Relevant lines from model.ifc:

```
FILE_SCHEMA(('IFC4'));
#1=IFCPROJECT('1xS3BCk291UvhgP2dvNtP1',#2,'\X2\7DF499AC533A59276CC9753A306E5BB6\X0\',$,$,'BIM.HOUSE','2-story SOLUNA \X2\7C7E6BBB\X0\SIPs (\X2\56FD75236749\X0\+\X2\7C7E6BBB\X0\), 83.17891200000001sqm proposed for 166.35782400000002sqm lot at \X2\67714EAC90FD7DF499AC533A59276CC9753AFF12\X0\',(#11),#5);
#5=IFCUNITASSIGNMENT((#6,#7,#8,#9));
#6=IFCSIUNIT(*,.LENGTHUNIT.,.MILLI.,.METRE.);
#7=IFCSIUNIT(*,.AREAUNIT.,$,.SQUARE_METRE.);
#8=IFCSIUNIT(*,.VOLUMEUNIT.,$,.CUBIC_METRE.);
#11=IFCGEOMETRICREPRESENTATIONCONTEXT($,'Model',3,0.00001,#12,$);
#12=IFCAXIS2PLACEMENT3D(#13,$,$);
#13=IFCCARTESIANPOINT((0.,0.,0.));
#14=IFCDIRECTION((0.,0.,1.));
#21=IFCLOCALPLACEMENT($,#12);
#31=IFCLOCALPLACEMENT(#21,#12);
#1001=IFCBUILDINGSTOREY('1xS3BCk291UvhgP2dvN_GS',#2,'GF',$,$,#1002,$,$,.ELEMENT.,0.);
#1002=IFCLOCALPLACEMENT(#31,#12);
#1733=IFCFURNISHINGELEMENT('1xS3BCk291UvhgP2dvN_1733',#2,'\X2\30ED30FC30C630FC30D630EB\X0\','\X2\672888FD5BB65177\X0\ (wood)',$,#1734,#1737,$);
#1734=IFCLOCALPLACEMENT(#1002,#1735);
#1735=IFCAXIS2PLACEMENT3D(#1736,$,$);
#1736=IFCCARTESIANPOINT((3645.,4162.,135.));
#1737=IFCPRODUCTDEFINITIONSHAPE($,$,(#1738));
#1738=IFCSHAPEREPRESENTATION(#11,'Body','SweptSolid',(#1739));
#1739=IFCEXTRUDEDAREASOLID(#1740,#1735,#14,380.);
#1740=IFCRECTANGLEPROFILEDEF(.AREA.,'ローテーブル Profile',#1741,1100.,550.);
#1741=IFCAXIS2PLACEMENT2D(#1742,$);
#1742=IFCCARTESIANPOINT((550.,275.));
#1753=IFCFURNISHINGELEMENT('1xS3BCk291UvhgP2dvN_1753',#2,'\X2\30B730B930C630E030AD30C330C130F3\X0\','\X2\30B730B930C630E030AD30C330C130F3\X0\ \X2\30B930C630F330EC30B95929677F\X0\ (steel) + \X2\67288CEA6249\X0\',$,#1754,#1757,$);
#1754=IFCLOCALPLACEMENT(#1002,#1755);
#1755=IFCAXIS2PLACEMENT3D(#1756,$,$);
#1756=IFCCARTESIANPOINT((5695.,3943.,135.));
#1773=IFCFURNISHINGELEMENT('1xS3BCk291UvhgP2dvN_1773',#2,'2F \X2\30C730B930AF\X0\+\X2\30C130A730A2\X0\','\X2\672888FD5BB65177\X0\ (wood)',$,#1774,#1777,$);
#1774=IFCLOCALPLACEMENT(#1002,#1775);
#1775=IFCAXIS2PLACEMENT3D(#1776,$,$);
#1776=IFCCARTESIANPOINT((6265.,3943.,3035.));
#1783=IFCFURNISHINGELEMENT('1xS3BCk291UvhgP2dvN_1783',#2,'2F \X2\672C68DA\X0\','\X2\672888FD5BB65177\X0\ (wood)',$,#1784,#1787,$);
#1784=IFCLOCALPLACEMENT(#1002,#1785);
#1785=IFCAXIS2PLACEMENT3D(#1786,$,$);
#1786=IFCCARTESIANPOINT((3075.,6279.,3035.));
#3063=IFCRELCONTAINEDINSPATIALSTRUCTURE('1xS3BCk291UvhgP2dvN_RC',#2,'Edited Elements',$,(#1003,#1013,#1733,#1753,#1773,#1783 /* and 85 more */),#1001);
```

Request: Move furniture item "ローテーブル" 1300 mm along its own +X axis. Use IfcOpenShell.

```python
import ifcopenshell
import ifcopenshell.api.geometry
import ifcopenshell.util.placement
import ifcopenshell.util.unit

model = ifcopenshell.open("model.ifc")
unit_scale = ifcopenshell.util.unit.calculate_unit_scale(model)

item = model.by_guid("1xS3BCk291UvhgP2dvN_1733")
matrix = ifcopenshell.util.placement.get_local_placement(item.ObjectPlacement)
matrix[:3, 3] += matrix[:3, 0] * 1.3 / unit_scale
ifcopenshell.api.geometry.edit_object_placement(model, product=item, matrix=matrix, is_si=False)

print(ifcopenshell.util.placement.get_local_placement(item.ObjectPlacement).round(3) + 0.0)

model.write("model_rev.ifc")
```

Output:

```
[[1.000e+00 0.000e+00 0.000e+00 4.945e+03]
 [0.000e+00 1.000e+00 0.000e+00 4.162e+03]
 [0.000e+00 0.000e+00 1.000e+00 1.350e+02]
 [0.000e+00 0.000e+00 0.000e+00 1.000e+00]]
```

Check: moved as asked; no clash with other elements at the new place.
